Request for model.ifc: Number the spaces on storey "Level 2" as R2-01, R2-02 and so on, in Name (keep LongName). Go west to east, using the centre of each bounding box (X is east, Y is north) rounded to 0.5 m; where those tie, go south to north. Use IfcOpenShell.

First a look at what the model holds.

```python
import ifcopenshell
import ifcopenshell.util.element
import ifcopenshell.util.placement

model = ifcopenshell.open("model.ifc")
print(model.schema)
storey = next(s for s in model.by_type("IfcBuildingStorey") if s.Name == "Level 2")
spaces = [e for e in ifcopenshell.util.element.get_decomposition(storey) if e.is_a("IfcSpace")]
for e in sorted(spaces, key=lambda e: e.id()):
    origin = ifcopenshell.util.placement.get_local_placement(e.ObjectPlacement)[:3, 3]
    print(e.id(), e.Name, e.LongName, origin.round(2) + 0.0, sep=" | ")
```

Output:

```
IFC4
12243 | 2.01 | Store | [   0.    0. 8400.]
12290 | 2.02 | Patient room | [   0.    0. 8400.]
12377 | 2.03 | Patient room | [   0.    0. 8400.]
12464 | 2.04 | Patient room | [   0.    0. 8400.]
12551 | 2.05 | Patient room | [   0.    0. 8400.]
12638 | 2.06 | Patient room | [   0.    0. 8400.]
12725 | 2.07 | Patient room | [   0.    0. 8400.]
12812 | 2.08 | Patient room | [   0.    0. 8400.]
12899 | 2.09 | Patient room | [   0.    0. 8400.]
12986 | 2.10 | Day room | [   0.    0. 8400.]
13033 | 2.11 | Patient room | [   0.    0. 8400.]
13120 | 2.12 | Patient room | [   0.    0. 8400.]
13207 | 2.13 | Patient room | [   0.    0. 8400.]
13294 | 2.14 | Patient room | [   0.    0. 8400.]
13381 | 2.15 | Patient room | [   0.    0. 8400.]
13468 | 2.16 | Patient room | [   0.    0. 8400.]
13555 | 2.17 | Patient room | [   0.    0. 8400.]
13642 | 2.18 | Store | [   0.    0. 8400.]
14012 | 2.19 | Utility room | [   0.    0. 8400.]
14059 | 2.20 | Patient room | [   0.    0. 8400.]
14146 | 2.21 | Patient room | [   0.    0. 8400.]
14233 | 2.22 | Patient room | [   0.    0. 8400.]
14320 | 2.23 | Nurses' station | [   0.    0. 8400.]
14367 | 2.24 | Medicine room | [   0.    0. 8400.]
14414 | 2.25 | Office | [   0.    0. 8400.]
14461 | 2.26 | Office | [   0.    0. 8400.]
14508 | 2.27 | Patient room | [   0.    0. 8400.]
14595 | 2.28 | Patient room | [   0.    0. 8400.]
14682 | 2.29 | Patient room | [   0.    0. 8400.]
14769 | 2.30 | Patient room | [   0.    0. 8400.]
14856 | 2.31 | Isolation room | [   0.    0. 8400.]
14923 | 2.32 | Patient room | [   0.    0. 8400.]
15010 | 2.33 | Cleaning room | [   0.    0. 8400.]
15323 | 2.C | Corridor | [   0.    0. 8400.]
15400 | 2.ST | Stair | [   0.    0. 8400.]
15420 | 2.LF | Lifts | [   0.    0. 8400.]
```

```python
import ifcopenshell
import ifcopenshell.geom
import ifcopenshell.util.element
import ifcopenshell.util.shape

model = ifcopenshell.open("model.ifc")
settings = ifcopenshell.geom.settings()
settings.set("use-world-coords", True)


def centre(element):
    shape = ifcopenshell.geom.create_shape(settings, element)
    return ifcopenshell.util.shape.get_bbox_centroid(shape.geometry)


storey = next(s for s in model.by_type("IfcBuildingStorey") if s.Name == "Level 2")
spaces = [e for e in ifcopenshell.util.element.get_decomposition(storey) if e.is_a("IfcSpace")]

# Insertion points can sit at a corner or the storey origin, so sort by the geometry (in metres).
centres = {e: centre(e) for e in spaces}
spaces.sort(key=lambda e: (round(centres[e][0] / 0.5), centres[e][1]))

for i, e in enumerate(spaces, start=1):
    number = f"R2-{i:02d}"
    e.Name = number
    print(e.id(), number)

model.write("model_edited.ifc")
```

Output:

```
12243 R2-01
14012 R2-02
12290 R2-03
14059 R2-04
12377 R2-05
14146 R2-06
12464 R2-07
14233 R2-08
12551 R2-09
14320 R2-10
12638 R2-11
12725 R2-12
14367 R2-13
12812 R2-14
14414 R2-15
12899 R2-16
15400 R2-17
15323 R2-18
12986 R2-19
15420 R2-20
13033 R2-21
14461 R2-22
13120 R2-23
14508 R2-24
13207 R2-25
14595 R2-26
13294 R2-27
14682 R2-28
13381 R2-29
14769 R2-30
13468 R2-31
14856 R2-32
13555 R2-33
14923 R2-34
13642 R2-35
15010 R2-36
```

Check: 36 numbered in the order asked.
